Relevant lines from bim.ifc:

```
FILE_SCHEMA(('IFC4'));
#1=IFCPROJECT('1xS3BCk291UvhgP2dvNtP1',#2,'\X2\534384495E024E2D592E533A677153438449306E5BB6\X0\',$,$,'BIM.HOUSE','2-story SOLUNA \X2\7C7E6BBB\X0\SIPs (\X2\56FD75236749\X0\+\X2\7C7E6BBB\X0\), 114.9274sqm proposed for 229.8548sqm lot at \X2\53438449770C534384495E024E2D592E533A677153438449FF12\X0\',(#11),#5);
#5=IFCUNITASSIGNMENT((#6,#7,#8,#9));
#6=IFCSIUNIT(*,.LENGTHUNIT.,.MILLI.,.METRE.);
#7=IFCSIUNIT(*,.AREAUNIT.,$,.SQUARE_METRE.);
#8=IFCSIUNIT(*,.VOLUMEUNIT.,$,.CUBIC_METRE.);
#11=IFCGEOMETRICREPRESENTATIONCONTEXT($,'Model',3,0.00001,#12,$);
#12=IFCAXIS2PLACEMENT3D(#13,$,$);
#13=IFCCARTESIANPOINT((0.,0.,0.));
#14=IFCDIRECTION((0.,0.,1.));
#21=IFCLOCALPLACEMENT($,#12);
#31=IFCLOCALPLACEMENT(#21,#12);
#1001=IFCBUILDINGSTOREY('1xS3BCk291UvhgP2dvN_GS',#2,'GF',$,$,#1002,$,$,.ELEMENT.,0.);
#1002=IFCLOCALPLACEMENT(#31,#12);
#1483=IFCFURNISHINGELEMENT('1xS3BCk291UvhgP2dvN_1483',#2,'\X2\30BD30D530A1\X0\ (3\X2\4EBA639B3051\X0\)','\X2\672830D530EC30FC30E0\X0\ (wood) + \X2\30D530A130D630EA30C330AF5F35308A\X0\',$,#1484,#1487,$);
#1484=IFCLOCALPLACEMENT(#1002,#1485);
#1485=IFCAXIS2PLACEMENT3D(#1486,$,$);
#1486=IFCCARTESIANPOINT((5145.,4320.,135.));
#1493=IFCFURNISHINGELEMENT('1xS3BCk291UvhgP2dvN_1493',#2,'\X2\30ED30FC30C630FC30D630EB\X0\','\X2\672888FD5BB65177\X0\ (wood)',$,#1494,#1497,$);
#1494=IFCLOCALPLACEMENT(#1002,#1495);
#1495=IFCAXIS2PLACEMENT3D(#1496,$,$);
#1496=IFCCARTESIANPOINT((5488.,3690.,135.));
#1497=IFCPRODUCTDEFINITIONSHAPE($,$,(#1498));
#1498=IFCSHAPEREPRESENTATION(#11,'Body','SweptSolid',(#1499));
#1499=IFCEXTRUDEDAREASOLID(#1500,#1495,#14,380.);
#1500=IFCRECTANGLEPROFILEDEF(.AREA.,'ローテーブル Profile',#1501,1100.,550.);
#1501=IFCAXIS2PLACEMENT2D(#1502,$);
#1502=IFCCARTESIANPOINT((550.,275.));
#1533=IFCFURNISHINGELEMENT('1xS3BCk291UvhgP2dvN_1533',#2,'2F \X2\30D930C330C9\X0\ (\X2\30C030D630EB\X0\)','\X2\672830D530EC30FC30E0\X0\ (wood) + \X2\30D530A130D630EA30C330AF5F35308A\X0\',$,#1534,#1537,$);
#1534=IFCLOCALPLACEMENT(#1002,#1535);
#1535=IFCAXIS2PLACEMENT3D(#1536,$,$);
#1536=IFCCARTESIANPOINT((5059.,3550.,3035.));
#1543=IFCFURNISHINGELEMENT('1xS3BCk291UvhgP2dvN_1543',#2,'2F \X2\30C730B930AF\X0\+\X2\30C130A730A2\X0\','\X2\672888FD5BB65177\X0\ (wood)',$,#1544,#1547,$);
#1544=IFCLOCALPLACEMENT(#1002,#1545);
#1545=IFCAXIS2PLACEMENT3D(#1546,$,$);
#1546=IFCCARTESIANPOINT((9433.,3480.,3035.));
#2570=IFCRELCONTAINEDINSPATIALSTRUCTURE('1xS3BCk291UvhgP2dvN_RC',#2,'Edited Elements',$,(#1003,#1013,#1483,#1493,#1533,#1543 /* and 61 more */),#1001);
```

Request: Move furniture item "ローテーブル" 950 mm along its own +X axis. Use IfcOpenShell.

```python
import ifcopenshell
import ifcopenshell.api.geometry
import ifcopenshell.util.placement

model = ifcopenshell.open("bim.ifc")

item = model.by_guid("1xS3BCk291UvhgP2dvN_1493")
matrix = ifcopenshell.util.placement.get_local_placement(item.ObjectPlacement)
matrix[:3, 3] += matrix[:3, 0] * 950.0
ifcopenshell.api.geometry.edit_object_placement(model, product=item, matrix=matrix, is_si=False)

print(ifcopenshell.util.placement.get_local_placement(item.ObjectPlacement).round(3) + 0.0)

model.write("bim_rev.ifc")
```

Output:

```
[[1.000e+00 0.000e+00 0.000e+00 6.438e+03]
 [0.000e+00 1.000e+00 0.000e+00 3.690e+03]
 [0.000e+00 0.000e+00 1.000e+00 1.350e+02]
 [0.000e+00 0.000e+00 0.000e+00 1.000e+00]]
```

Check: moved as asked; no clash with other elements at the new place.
